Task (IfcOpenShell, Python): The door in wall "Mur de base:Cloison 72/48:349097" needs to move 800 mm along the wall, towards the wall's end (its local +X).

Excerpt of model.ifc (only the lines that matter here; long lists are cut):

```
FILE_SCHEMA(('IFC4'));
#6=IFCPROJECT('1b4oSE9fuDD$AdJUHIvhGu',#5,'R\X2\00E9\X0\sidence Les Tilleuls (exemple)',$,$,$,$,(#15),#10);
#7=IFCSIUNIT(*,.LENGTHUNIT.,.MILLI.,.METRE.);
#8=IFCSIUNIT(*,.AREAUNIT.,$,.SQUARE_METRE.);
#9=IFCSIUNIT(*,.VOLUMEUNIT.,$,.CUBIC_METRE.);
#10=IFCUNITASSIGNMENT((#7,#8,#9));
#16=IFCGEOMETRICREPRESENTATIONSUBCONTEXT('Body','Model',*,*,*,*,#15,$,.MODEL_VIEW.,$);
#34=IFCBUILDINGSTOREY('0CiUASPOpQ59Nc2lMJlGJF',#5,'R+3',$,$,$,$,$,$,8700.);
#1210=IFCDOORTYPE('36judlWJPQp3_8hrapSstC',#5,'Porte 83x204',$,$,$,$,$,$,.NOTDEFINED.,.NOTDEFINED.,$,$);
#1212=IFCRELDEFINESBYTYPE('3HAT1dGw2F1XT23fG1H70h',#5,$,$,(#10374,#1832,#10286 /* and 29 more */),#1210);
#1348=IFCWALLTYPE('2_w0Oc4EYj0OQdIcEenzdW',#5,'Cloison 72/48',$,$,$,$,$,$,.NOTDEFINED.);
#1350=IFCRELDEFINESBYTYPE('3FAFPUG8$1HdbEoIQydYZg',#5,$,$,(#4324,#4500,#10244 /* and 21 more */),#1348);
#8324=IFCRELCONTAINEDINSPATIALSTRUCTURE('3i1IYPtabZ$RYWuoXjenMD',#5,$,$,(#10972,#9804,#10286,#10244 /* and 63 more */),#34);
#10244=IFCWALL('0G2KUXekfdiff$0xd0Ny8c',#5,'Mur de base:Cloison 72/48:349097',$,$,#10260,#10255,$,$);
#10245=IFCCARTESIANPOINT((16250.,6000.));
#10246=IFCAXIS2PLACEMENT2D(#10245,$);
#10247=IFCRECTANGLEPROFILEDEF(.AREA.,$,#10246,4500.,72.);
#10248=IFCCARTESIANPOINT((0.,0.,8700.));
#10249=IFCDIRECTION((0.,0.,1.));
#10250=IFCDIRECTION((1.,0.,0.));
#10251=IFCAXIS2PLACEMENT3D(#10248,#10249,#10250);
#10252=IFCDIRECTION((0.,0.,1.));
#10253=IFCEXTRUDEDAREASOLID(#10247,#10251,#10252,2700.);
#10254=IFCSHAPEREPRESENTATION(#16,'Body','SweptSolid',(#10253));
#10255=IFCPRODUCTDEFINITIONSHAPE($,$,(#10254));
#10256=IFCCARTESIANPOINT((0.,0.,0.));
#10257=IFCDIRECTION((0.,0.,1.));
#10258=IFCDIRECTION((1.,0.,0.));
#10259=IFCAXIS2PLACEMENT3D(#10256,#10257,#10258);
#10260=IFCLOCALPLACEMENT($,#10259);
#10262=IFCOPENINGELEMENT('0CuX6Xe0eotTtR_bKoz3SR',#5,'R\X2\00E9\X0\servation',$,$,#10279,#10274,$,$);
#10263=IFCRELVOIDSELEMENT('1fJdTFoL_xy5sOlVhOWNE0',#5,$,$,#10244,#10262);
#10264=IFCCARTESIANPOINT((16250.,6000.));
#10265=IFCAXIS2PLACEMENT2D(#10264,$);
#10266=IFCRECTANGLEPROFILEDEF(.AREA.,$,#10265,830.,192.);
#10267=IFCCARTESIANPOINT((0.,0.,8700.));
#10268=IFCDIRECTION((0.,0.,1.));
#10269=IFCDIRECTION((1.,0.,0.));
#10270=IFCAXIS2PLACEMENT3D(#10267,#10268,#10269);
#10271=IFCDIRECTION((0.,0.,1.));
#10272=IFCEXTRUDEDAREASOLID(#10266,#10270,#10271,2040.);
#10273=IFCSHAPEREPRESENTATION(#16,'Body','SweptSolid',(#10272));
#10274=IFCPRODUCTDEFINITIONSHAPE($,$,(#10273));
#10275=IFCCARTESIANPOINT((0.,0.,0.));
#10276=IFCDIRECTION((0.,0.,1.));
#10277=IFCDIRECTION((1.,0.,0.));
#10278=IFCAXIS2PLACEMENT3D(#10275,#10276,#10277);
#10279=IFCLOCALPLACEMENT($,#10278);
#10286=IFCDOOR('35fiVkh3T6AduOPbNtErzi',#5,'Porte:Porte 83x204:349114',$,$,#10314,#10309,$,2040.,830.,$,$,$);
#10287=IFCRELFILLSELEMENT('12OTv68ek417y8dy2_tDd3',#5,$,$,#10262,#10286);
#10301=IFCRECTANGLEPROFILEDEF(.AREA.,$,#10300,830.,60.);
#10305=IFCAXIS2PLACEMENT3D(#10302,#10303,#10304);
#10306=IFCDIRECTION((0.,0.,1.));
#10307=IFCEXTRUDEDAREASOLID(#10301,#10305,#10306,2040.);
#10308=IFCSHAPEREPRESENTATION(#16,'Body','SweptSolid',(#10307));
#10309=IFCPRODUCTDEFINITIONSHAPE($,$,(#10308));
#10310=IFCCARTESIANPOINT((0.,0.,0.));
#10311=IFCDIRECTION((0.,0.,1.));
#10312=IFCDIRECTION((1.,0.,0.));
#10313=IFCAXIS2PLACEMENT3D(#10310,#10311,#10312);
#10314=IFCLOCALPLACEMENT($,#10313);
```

```python
import ifcopenshell
import ifcopenshell.api.geometry
import ifcopenshell.util.placement
import ifcopenshell.util.unit

model = ifcopenshell.open("model.ifc")
unit_scale = ifcopenshell.util.unit.calculate_unit_scale(model)

door = model.by_guid("35fiVkh3T6AduOPbNtErzi")
opening = door.FillsVoids[0].RelatingOpeningElement
wall = opening.VoidsElements[0].RelatingBuildingElement

wall_matrix = ifcopenshell.util.placement.get_local_placement(wall.ObjectPlacement)
shift = wall_matrix[:3, 0] * 0.8 / unit_scale
before = ifcopenshell.util.placement.get_local_placement(door.ObjectPlacement)[:3, 3].copy()

# The door is not placed relative to its opening, so move both.
for product in (opening, door):
    matrix = ifcopenshell.util.placement.get_local_placement(product.ObjectPlacement)
    matrix[:3, 3] += shift
    ifcopenshell.api.geometry.edit_object_placement(model, product=product, matrix=matrix, is_si=False)

after = ifcopenshell.util.placement.get_local_placement(door.ObjectPlacement)[:3, 3]
print("door moved by", (after - before).round(3) + 0.0)

model.write("model-out.ifc")
```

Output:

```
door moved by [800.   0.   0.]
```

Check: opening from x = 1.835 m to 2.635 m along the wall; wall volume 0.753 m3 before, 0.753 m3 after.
